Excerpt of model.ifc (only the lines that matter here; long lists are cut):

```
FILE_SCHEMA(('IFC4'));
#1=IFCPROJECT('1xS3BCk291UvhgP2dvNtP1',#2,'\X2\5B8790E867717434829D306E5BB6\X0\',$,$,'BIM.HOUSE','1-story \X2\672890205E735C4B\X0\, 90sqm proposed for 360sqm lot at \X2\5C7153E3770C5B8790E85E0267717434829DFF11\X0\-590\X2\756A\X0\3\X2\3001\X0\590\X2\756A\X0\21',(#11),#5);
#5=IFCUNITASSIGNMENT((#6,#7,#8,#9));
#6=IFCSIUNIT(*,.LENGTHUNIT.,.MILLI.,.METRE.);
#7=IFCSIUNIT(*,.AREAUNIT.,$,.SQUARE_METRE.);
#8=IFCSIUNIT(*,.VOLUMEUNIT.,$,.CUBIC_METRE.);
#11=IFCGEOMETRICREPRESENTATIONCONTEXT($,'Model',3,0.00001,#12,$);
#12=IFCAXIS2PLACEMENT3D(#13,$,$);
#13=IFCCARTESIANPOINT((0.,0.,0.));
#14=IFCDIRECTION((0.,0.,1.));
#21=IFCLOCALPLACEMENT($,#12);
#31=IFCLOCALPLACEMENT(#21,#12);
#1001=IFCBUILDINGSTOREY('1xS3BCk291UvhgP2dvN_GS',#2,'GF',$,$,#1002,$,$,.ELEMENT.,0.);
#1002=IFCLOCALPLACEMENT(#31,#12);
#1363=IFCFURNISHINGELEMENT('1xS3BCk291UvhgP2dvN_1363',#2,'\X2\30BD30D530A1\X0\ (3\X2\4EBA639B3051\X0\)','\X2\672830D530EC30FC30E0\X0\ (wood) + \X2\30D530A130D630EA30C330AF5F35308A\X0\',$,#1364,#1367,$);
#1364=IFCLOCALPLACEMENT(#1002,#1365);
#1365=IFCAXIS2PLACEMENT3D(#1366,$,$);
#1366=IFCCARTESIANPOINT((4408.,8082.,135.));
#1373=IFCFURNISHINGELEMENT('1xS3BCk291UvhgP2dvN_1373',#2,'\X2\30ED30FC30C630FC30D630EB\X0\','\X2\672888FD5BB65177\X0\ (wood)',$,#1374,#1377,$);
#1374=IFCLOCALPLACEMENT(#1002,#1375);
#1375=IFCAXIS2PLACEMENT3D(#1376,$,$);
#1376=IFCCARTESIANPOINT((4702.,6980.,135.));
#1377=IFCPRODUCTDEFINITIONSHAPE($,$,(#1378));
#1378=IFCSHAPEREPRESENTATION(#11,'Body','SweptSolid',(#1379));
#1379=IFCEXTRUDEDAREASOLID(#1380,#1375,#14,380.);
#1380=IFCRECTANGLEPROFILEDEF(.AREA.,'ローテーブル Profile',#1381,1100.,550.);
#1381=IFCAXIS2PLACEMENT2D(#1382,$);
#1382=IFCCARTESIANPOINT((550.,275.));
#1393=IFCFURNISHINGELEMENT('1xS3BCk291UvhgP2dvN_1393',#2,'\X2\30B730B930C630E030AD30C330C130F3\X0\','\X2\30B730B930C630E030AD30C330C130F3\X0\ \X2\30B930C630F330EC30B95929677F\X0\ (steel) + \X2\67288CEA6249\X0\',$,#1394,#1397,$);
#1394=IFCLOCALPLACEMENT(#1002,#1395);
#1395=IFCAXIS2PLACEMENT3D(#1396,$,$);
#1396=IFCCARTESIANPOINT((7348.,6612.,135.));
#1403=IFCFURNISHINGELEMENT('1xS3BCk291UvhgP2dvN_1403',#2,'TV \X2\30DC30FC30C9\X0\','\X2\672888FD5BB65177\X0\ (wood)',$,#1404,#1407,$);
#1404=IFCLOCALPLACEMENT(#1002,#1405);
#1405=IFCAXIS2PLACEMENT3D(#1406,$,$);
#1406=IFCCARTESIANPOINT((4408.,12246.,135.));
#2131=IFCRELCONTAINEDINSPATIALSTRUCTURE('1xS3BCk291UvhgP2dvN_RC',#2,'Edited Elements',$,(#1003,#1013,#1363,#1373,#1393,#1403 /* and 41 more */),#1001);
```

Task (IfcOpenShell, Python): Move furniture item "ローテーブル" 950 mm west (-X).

```python
import ifcopenshell
import ifcopenshell.api.geometry
import ifcopenshell.util.placement
import ifcopenshell.util.unit

model = ifcopenshell.open("model.ifc")
unit_scale = ifcopenshell.util.unit.calculate_unit_scale(model)

item = model.by_guid("1xS3BCk291UvhgP2dvN_1373")
matrix = ifcopenshell.util.placement.get_local_placement(item.ObjectPlacement)
matrix[0, 3] -= 0.95 / unit_scale
ifcopenshell.api.geometry.edit_object_placement(model, product=item, matrix=matrix, is_si=False)

print(ifcopenshell.util.placement.get_local_placement(item.ObjectPlacement).round(3) + 0.0)

model.write("model_edited.ifc")
```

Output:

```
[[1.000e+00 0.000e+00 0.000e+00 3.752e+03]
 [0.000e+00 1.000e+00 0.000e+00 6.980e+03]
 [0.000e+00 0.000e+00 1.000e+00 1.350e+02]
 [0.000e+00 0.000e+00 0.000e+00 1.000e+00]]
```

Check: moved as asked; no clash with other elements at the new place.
